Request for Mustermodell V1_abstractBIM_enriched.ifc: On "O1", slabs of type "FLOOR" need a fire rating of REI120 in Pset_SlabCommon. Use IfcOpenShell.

First a look at what the model holds.

```python
import ifcopenshell
import ifcopenshell.util.element

model = ifcopenshell.open("Mustermodell V1_abstractBIM_enriched.ifc")
print(model.schema)
storey = next(s for s in model.by_type("IfcBuildingStorey") if s.Name == "O1")
slabs = [e for e in ifcopenshell.util.element.get_decomposition(storey) if e.is_a("IfcSlab")]
seen = {}
for e in slabs:
    element_type = ifcopenshell.util.element.get_type(e)
    key = (element_type.Name if element_type != e and element_type else None, ifcopenshell.util.element.get_pset(e, "Pset_SlabCommon", "FireRating"))
    seen[key] = seen.get(key, 0) + 1
for (name, value), count in sorted(seen.items(), key=str):
    print(count, "x", name, "|", value)
```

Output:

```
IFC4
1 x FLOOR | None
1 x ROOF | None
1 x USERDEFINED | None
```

```python
import ifcopenshell
import ifcopenshell.api.pset
import ifcopenshell.util.element

model = ifcopenshell.open("Mustermodell V1_abstractBIM_enriched.ifc")

storey = next(s for s in model.by_type("IfcBuildingStorey") if s.Name == "O1")
slabs = [e for e in ifcopenshell.util.element.get_decomposition(storey) if e.is_a("IfcSlab")]

count = 0
for e in slabs:
    element_type = ifcopenshell.util.element.get_type(e)
    if element_type in (None, e) or element_type.Name != "FLOOR":
        continue
    # add_pset returns the element's existing set when there is one.
    pset = ifcopenshell.api.pset.add_pset(model, product=e, name="Pset_SlabCommon")
    ifcopenshell.api.pset.edit_pset(model, pset=pset, properties={"FireRating": "REI120"})
    count += 1

print(count, "slabs updated")

model.write("Mustermodell V1_abstractBIM_enriched_edited.ifc")
```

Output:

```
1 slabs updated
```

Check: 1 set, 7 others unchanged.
